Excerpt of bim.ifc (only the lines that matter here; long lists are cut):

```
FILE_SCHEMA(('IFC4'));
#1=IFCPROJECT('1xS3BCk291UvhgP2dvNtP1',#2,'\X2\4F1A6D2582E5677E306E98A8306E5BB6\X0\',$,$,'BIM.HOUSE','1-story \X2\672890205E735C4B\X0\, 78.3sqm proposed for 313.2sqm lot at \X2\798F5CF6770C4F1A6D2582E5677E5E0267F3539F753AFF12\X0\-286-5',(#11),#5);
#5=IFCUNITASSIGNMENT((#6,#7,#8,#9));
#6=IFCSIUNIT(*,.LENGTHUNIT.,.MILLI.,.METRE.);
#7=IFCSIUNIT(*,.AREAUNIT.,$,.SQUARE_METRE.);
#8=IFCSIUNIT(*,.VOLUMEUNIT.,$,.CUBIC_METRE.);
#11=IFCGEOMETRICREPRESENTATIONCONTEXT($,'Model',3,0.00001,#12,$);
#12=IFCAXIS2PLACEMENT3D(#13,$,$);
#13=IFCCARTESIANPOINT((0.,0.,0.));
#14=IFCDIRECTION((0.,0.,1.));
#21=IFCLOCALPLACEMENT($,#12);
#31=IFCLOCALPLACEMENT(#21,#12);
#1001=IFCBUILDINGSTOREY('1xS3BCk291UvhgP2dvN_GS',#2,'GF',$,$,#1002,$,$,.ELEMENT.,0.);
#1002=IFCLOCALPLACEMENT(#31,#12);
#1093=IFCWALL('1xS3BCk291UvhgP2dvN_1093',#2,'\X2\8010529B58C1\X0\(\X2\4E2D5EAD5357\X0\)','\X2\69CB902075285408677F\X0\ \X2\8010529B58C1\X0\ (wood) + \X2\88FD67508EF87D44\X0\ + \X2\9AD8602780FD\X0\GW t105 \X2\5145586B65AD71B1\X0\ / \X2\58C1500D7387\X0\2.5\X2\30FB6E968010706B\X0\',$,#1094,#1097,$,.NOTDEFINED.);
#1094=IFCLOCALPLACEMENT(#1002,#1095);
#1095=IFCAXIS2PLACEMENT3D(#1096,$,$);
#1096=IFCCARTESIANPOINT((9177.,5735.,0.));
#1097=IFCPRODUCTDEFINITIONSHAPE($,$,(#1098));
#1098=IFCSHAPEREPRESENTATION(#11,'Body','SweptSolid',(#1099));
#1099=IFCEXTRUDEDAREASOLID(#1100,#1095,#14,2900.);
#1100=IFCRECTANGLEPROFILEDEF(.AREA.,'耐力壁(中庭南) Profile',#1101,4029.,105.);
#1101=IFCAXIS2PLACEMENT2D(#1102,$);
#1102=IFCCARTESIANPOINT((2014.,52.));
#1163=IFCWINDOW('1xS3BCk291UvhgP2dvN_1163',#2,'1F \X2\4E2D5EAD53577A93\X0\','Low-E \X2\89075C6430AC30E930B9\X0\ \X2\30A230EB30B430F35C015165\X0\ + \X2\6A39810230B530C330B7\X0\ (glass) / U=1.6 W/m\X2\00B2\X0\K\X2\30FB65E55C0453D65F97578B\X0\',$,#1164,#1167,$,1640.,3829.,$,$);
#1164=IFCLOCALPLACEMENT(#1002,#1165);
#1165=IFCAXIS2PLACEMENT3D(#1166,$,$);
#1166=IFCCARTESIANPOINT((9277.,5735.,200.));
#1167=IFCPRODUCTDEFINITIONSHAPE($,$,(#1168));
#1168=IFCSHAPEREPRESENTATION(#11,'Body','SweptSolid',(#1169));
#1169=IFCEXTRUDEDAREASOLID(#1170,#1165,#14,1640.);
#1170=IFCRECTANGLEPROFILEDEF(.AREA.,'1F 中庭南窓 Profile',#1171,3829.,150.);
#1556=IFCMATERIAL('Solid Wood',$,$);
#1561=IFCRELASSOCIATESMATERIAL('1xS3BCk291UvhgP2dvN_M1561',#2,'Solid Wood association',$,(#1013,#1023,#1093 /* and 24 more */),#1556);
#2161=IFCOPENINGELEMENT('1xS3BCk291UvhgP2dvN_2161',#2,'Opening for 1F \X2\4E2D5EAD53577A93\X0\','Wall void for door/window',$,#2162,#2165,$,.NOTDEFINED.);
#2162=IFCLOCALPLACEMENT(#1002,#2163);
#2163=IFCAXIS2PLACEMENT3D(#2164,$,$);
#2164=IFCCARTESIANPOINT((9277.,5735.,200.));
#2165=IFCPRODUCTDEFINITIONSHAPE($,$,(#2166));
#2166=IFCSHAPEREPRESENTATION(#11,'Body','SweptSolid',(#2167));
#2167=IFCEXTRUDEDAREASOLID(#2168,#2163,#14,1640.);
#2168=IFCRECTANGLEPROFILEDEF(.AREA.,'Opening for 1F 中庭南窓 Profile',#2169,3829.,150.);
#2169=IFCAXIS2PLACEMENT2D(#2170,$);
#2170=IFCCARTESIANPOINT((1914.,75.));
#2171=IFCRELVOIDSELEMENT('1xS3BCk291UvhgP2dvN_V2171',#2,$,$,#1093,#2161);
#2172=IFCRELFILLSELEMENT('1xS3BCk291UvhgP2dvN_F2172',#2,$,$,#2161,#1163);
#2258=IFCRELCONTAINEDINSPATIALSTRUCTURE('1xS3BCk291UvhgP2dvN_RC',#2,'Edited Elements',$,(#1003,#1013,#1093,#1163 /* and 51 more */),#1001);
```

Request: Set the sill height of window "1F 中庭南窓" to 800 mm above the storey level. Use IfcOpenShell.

```python
import numpy as np
import ifcopenshell
import ifcopenshell.api.geometry
import ifcopenshell.geom
import ifcopenshell.util.element
import ifcopenshell.util.placement
import ifcopenshell.util.shape
import ifcopenshell.util.unit

model = ifcopenshell.open("bim.ifc")
unit_scale = ifcopenshell.util.unit.calculate_unit_scale(model)

window = model.by_guid("1xS3BCk291UvhgP2dvN_1163")
opening = window.FillsVoids[0].RelatingOpeningElement
storey = ifcopenshell.util.element.get_container(window, ifc_class="IfcBuildingStorey")
level = ifcopenshell.util.placement.get_local_placement(storey.ObjectPlacement)[2, 3]

# The opening's origin need not be at the sill, so measure its lowest point.
shape = ifcopenshell.geom.create_shape(ifcopenshell.geom.settings(), opening)
bottom = ifcopenshell.util.shape.get_shape_bottom_elevation(shape, shape.geometry) / unit_scale
dz = level + 0.8 / unit_scale - bottom

shift = np.array([0.0, 0.0, dz])
# The window is not placed relative to its opening, so move both.
for product in (opening, window):
    matrix = ifcopenshell.util.placement.get_local_placement(product.ObjectPlacement)
    matrix[:3, 3] += shift
    ifcopenshell.api.geometry.edit_object_placement(model, product=product, matrix=matrix, is_si=False)

print(f"moved by {dz * unit_scale:+.3f} m")

model.write("bim-out.ifc")
```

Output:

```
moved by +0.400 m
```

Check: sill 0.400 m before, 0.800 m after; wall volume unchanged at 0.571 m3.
